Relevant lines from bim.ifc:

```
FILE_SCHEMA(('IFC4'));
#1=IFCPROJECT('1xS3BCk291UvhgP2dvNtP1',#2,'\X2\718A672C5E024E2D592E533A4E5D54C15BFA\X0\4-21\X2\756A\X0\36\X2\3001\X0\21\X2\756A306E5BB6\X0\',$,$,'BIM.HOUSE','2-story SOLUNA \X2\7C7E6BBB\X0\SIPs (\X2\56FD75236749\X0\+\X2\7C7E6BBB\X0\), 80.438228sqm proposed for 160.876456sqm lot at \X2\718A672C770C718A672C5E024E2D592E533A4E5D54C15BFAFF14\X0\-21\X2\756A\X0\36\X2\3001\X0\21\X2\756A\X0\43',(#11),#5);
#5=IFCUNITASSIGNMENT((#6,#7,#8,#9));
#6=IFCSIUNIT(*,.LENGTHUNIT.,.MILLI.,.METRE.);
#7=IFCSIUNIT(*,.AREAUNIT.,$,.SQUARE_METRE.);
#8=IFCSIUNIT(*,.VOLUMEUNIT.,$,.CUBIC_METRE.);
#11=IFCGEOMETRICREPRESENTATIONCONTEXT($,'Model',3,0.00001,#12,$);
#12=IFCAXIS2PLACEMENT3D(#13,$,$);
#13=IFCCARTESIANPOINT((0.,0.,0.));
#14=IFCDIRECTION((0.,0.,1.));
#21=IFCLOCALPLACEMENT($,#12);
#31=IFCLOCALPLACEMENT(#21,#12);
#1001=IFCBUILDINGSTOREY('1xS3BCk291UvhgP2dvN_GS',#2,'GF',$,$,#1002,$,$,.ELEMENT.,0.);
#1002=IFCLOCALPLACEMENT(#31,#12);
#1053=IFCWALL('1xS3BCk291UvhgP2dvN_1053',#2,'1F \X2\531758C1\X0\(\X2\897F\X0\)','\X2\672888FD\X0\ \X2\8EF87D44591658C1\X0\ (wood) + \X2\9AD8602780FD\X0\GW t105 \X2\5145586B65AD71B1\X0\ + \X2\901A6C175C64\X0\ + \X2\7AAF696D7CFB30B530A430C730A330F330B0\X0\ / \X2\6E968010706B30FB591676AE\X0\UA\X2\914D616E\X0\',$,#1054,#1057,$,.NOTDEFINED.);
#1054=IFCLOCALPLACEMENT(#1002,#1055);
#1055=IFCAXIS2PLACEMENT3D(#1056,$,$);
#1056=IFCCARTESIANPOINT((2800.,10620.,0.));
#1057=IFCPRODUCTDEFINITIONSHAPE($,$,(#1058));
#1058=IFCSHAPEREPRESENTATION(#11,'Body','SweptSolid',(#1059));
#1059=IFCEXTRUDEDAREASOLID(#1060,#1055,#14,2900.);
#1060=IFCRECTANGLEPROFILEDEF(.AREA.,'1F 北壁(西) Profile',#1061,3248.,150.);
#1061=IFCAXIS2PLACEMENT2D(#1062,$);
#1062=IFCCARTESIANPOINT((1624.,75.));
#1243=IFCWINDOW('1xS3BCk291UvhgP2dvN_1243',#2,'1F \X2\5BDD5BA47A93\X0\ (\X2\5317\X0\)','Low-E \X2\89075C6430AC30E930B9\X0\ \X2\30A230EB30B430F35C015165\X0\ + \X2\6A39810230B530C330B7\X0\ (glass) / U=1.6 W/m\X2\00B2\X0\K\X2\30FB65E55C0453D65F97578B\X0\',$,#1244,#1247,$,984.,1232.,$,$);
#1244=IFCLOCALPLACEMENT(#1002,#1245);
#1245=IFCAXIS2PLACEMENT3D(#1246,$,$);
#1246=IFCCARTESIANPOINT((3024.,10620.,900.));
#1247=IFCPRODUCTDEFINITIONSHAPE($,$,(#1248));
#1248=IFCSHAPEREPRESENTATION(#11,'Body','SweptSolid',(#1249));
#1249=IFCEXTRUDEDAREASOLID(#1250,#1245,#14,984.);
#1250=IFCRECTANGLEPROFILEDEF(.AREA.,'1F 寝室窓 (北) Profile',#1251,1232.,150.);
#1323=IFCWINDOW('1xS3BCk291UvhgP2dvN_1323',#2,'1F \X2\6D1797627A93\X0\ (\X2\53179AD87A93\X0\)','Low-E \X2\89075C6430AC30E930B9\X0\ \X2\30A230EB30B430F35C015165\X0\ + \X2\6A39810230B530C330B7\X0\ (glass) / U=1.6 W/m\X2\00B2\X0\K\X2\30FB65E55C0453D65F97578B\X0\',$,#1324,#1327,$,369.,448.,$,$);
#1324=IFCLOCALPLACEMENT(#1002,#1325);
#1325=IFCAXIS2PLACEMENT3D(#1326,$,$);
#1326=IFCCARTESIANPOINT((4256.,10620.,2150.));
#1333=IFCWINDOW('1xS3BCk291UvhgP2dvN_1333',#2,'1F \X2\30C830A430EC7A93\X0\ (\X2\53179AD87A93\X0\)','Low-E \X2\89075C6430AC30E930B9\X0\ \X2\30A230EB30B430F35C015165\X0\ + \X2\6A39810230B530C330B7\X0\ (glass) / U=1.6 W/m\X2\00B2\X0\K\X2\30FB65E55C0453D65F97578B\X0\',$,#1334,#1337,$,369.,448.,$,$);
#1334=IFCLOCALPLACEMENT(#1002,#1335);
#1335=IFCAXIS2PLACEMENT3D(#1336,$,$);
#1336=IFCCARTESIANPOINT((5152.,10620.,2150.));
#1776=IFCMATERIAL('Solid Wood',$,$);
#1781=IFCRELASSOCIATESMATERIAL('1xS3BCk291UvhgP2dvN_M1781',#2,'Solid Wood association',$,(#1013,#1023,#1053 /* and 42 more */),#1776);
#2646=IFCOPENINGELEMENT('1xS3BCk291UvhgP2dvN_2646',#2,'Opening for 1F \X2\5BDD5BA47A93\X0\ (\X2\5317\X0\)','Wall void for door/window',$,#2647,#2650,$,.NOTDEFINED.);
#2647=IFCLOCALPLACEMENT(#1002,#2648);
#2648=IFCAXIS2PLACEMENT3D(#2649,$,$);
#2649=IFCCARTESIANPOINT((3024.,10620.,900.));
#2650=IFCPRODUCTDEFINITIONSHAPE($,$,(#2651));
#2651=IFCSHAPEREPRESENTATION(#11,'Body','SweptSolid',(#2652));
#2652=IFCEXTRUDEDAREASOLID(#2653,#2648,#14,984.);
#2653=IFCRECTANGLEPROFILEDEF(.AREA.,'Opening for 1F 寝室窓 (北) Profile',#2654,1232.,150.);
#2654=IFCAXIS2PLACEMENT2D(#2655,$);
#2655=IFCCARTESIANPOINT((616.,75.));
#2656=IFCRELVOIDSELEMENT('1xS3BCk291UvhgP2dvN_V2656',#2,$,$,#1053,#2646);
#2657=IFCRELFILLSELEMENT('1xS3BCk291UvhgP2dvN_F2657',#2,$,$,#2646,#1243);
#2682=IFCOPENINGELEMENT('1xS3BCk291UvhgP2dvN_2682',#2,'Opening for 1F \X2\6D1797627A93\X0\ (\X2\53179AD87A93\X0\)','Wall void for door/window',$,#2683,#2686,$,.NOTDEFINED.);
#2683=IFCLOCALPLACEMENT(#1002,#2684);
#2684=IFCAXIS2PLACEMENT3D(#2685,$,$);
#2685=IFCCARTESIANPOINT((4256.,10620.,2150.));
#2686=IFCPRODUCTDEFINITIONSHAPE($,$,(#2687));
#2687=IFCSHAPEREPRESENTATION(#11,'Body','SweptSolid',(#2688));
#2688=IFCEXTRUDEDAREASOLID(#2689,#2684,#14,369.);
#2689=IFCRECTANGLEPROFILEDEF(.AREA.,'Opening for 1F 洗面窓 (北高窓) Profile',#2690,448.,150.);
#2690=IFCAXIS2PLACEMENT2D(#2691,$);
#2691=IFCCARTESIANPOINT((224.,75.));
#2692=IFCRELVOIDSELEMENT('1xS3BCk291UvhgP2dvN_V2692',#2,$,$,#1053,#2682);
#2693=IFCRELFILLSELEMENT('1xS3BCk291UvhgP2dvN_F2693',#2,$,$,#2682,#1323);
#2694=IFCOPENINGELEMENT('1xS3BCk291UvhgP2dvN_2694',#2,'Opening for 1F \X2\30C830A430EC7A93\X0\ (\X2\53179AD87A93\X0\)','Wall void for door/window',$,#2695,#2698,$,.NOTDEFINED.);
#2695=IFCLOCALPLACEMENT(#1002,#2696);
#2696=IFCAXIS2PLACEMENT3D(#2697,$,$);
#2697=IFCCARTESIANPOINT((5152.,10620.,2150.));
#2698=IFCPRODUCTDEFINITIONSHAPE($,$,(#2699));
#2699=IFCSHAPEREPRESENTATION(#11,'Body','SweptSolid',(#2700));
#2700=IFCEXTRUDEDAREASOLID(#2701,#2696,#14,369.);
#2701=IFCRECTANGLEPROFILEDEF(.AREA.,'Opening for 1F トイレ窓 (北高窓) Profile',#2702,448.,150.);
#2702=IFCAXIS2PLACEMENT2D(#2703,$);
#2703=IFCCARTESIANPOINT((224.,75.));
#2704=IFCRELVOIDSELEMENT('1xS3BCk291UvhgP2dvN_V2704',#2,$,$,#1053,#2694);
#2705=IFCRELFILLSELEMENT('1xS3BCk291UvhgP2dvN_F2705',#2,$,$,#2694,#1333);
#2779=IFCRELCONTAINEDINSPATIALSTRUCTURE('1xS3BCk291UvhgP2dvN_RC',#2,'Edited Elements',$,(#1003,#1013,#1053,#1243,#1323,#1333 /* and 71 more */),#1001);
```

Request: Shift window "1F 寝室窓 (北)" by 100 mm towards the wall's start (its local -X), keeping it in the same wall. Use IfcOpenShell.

```python
import ifcopenshell
import ifcopenshell.api.geometry
import ifcopenshell.util.placement

model = ifcopenshell.open("bim.ifc")

window = model.by_guid("1xS3BCk291UvhgP2dvN_1243")
opening = window.FillsVoids[0].RelatingOpeningElement
wall = opening.VoidsElements[0].RelatingBuildingElement

wall_matrix = ifcopenshell.util.placement.get_local_placement(wall.ObjectPlacement)
shift = wall_matrix[:3, 0] * -100.0
before = ifcopenshell.util.placement.get_local_placement(window.ObjectPlacement)[:3, 3].copy()

# The window is not placed relative to its opening, so move both.
for product in (opening, window):
    matrix = ifcopenshell.util.placement.get_local_placement(product.ObjectPlacement)
    matrix[:3, 3] += shift
    ifcopenshell.api.geometry.edit_object_placement(model, product=product, matrix=matrix, is_si=False)

after = ifcopenshell.util.placement.get_local_placement(window.ObjectPlacement)[:3, 3]
print("window moved by", (after - before).round(3) + 0.0)

model.write("bim_edited.ifc")
```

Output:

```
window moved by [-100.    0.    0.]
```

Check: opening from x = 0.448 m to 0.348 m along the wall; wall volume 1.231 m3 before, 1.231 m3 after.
